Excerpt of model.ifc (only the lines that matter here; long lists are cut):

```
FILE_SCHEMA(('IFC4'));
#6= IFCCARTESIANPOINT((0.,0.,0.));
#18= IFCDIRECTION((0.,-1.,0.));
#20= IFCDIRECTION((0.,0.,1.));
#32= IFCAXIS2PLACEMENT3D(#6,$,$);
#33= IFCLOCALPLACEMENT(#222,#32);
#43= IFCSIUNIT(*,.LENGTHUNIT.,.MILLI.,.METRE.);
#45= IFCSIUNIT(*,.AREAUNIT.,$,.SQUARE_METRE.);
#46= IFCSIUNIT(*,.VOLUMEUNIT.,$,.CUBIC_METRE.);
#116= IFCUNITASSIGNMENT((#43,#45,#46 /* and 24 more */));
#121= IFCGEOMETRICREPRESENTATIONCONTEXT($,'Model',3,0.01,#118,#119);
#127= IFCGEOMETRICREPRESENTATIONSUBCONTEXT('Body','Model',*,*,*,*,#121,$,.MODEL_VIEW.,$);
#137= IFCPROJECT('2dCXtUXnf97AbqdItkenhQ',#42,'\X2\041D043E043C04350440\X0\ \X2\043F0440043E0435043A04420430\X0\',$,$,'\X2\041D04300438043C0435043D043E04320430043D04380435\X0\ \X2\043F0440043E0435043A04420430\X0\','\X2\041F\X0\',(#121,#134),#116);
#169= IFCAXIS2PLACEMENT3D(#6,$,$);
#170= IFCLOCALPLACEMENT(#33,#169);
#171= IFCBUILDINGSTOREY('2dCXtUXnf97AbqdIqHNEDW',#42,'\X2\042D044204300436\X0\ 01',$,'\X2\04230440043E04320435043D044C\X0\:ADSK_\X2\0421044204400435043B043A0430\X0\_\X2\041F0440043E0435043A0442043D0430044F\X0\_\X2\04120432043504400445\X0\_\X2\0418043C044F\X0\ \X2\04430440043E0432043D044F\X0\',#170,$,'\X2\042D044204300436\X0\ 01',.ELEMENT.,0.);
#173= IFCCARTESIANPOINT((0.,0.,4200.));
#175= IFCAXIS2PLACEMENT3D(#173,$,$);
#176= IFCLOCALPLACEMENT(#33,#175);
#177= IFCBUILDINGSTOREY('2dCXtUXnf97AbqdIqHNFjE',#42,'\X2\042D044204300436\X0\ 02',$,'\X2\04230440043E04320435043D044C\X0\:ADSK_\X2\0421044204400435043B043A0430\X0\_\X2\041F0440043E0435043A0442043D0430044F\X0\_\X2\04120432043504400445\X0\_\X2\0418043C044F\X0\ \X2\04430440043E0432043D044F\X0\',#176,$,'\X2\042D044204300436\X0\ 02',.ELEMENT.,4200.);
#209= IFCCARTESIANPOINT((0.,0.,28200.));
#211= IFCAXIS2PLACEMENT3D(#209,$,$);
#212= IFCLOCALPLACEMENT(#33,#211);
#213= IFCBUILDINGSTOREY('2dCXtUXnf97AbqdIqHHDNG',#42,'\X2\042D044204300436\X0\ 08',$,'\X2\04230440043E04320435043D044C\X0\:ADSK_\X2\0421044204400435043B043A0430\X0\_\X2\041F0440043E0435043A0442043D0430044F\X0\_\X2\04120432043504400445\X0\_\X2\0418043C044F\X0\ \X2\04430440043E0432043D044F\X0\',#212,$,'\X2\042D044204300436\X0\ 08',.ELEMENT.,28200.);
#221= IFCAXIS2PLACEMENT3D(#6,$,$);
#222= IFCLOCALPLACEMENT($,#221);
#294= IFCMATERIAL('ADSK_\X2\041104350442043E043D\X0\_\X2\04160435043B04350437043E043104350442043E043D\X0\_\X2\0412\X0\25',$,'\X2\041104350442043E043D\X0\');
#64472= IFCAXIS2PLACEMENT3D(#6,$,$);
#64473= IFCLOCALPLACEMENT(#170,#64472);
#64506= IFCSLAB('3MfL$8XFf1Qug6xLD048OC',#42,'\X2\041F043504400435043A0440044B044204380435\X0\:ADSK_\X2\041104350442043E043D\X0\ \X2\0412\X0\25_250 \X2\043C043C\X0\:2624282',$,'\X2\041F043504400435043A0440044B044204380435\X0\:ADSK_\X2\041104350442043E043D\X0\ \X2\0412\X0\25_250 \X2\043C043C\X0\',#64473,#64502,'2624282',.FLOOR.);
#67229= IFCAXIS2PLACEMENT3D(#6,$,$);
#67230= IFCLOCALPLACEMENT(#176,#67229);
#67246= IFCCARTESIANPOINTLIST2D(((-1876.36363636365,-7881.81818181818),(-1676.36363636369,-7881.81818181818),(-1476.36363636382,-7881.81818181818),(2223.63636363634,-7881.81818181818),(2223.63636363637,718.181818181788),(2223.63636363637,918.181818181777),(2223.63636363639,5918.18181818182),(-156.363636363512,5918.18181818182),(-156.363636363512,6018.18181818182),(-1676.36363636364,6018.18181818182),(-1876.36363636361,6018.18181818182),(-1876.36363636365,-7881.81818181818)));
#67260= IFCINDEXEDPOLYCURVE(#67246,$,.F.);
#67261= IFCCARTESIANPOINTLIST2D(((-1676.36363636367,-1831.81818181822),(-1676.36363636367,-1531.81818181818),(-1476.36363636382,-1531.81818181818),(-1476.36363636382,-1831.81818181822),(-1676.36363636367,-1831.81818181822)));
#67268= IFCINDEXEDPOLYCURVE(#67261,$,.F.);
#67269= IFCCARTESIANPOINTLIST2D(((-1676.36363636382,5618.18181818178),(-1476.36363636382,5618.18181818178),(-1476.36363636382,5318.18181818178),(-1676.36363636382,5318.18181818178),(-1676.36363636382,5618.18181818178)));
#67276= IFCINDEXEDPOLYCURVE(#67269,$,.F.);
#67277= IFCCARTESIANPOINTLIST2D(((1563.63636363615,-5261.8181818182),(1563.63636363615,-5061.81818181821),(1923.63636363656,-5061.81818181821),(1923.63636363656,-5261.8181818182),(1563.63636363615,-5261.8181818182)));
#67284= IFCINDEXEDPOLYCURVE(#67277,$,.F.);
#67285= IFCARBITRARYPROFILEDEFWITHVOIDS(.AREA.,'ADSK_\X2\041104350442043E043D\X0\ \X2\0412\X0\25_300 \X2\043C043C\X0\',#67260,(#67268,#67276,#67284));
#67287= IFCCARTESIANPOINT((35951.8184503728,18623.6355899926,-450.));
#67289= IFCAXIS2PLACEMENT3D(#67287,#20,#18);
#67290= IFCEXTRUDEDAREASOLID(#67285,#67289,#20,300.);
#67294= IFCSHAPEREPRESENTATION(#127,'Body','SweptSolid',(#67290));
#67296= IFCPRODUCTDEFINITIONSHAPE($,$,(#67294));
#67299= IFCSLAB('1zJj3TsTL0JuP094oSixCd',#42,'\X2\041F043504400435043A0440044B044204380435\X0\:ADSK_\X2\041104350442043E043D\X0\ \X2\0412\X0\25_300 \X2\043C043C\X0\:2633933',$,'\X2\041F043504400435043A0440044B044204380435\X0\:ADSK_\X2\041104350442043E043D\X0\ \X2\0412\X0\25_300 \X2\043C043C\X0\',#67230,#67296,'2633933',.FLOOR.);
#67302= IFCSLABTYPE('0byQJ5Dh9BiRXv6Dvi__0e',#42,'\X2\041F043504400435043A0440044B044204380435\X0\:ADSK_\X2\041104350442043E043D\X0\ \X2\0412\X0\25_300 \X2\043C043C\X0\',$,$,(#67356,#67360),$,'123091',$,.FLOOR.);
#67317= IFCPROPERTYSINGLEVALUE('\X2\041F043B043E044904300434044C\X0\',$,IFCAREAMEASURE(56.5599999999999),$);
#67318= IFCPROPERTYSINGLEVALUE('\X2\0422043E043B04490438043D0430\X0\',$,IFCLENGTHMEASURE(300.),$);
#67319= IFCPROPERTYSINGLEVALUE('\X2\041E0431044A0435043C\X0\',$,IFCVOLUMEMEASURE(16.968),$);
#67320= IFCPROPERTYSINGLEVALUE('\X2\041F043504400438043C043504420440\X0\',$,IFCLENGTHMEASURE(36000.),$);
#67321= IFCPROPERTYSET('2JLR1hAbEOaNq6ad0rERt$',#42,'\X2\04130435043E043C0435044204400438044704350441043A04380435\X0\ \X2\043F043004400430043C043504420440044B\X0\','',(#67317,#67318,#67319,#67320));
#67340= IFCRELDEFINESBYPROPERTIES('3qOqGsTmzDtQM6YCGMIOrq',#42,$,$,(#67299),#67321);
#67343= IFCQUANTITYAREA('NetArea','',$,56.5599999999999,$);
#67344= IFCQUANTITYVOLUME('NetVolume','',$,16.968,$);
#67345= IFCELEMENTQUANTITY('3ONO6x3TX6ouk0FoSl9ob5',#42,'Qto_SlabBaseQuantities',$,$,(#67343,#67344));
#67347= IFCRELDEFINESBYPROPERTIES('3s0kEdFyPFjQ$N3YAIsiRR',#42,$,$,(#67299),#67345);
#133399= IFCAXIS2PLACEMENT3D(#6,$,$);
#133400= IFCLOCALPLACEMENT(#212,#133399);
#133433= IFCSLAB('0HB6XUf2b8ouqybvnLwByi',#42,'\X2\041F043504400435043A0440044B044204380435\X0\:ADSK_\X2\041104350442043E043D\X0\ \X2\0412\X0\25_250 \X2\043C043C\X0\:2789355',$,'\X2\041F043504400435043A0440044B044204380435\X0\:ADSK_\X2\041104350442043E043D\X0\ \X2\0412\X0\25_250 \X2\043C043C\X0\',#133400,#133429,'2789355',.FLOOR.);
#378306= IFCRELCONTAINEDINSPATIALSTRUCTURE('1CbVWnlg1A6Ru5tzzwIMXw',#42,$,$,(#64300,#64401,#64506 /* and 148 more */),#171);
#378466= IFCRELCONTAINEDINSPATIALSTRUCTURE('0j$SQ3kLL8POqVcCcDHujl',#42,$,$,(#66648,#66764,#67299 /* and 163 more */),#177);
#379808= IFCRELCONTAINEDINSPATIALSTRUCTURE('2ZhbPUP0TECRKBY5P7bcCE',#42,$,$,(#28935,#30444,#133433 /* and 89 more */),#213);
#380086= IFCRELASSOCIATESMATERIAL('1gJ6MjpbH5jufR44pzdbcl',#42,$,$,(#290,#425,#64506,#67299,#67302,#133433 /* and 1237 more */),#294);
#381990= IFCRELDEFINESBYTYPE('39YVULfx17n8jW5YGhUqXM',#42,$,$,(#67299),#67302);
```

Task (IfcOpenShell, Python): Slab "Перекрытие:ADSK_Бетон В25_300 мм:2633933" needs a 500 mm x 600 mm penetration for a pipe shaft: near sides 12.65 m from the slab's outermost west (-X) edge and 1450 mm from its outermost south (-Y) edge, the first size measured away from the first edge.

```python
import numpy as np
import ifcopenshell
import ifcopenshell.api.feature
import ifcopenshell.api.geometry
import ifcopenshell.api.pset
import ifcopenshell.api.root
import ifcopenshell.geom
import ifcopenshell.util.element
import ifcopenshell.util.placement
import ifcopenshell.util.representation
import ifcopenshell.util.shape
import ifcopenshell.util.unit

model = ifcopenshell.open("model.ifc")
unit_scale = ifcopenshell.util.unit.calculate_unit_scale(model)
area_scale = ifcopenshell.util.unit.calculate_unit_scale(model, "AREAUNIT")
volume_scale = ifcopenshell.util.unit.calculate_unit_scale(model, "VOLUMEUNIT")
settings = ifcopenshell.geom.settings()


def volume(element):
    """Net volume in cubic metres, openings subtracted."""
    shape = ifcopenshell.geom.create_shape(settings, element)
    return ifcopenshell.util.shape.get_volume(shape.geometry)


slab = model.by_guid("1zJj3TsTL0JuP094oSixCd")
before = volume(slab)

# Extent in the slab's own axes, in metres. The edges named are its -X and -Y sides.
slab_shape = ifcopenshell.geom.create_shape(settings, slab)
vertices = ifcopenshell.util.shape.get_vertices(slab_shape.geometry)
x_min, y_min, bottom = vertices.min(axis=0)
top = vertices[:, 2].max()

opening = ifcopenshell.api.root.create_entity(model, ifc_class="IfcOpeningElement", name="Pipe shaft opening", predefined_type="OPENING")
context = ifcopenshell.util.representation.get_context(model, "Model", "Body", "MODEL_VIEW")
width, depth = 0.5, 0.6
outline = [(0.0, 0.0), (width, 0.0), (width, depth), (0.0, depth), (0.0, 0.0)]
# Overshoot both faces by 50 mm so the cut is clean.
shape = ifcopenshell.api.geometry.add_slab_representation(
    model, context=context, depth=top - bottom + 0.1, polyline=outline
)
ifcopenshell.api.geometry.assign_representation(model, product=opening, representation=shape)

matrix = ifcopenshell.util.placement.get_local_placement(slab.ObjectPlacement)
matrix[:, 3] = matrix @ np.append(np.array([x_min + 12.65, y_min + 1.45, bottom - 0.05]) / unit_scale, 1.0)
ifcopenshell.api.geometry.edit_object_placement(model, product=opening, matrix=matrix, is_si=False)
ifcopenshell.api.feature.add_feature(model, feature=opening, element=slab)

after = volume(slab)

# Update the slab's stored quantities.
pset = model.by_id(ifcopenshell.util.element.get_pset(slab, "Геометрические параметры", should_inherit=False)["id"])
ifcopenshell.api.pset.edit_pset(model, pset=pset, properties={
    "Площадь": model.create_entity("IfcAreaMeasure", after / (top - bottom) / area_scale),
    "Объем": model.create_entity("IfcVolumeMeasure", after / volume_scale),
})
qto = model.by_id(ifcopenshell.util.element.get_pset(slab, "Qto_SlabBaseQuantities", should_inherit=False)["id"])
ifcopenshell.api.pset.edit_qto(model, qto=qto, properties={
    "NetArea": after / (top - bottom) / area_scale,
    "NetVolume": after / volume_scale,
})

print(f"slab volume {before:.3f} -> {after:.3f} m3")

model.write("model_v2.ifc")
```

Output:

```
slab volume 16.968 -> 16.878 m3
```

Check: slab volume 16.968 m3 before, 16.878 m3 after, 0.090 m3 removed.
